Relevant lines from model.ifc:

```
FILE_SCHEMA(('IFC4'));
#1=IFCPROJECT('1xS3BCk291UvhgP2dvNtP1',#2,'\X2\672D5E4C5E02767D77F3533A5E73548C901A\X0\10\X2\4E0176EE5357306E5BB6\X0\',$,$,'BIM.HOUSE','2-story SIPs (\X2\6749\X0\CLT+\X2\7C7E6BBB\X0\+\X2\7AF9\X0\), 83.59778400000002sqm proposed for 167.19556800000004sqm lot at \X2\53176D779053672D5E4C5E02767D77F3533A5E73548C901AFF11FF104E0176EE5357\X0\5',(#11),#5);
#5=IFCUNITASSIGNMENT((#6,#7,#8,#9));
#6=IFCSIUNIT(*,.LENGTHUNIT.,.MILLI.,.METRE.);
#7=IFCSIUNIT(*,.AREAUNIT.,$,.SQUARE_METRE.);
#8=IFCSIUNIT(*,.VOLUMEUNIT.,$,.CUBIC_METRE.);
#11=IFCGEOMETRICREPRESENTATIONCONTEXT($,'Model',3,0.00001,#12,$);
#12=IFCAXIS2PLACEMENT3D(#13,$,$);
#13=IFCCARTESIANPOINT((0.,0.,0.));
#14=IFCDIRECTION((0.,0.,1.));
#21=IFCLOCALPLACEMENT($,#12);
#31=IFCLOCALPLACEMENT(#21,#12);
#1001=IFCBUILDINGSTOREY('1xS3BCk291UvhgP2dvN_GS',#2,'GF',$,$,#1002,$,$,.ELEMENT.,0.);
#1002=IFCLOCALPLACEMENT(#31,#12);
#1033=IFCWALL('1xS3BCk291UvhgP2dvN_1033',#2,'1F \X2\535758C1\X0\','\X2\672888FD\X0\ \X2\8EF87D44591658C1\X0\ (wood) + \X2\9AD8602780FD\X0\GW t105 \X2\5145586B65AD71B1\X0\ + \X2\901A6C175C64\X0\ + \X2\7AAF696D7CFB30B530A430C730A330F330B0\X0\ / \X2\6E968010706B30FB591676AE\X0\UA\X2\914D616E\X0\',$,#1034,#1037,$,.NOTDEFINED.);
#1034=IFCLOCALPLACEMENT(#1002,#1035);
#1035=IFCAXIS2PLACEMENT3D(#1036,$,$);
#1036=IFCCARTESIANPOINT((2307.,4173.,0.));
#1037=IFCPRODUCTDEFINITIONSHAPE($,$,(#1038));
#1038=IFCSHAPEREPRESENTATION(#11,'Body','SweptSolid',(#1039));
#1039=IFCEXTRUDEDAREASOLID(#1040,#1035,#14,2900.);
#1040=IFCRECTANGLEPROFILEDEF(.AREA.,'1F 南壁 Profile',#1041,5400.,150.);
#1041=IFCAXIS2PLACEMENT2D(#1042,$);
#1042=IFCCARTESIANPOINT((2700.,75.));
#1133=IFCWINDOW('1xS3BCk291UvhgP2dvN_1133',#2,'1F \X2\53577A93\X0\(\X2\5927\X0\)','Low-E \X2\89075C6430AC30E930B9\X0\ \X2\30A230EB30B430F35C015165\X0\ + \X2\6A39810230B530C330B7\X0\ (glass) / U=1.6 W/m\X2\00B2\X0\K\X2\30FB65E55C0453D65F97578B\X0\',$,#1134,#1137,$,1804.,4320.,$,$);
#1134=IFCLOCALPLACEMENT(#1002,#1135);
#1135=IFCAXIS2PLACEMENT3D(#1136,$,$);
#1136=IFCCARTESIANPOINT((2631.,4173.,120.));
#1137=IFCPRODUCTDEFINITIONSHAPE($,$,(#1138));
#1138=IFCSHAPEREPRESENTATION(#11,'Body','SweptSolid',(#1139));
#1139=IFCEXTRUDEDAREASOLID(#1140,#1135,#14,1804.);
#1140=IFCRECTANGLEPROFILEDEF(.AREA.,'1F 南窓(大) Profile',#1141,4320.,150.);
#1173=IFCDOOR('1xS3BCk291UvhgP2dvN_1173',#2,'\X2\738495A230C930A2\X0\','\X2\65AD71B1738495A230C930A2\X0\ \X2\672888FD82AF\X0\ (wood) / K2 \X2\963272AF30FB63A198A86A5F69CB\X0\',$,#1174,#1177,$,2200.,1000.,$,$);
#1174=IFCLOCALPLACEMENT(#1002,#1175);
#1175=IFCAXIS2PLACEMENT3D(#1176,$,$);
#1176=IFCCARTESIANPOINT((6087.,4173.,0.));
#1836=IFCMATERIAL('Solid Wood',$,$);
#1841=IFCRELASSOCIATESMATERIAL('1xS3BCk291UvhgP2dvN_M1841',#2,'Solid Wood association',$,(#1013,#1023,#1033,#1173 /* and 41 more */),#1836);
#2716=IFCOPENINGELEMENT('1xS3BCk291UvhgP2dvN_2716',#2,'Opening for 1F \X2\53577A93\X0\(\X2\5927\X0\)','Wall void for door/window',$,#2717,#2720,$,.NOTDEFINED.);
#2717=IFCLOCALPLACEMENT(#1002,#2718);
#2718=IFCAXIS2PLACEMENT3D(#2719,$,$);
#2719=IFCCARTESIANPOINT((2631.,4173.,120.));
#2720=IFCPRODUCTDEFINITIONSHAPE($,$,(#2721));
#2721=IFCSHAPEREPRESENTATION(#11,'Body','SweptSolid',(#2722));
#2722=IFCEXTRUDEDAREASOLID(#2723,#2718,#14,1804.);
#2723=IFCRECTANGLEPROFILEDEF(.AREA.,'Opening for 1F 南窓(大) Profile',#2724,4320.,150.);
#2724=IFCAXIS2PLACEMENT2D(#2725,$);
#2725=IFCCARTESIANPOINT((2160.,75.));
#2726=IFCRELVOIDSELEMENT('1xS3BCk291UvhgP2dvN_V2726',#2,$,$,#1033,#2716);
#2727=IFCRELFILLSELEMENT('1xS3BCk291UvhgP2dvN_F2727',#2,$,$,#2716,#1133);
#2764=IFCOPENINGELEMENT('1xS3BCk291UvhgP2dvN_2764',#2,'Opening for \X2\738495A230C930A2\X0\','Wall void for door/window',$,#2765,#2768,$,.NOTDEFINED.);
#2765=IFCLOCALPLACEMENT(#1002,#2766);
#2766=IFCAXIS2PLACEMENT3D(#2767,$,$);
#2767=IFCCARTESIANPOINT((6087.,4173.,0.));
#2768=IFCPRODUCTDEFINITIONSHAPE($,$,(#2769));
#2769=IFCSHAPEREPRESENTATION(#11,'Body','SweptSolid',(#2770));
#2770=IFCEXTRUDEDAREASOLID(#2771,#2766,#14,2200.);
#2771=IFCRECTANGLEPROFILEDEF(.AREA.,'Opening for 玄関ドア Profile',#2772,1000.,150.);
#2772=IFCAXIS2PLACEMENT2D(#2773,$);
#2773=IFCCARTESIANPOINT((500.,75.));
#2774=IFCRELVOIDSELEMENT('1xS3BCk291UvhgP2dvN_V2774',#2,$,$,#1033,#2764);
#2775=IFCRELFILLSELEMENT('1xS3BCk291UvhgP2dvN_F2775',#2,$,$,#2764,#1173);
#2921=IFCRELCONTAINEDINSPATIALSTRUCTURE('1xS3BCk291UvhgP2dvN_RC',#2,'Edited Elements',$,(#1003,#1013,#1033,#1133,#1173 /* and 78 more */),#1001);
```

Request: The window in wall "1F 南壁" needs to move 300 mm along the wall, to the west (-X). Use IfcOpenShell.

```python
import ifcopenshell
import ifcopenshell.api.geometry
import ifcopenshell.util.placement
import ifcopenshell.util.unit

model = ifcopenshell.open("model.ifc")
unit_scale = ifcopenshell.util.unit.calculate_unit_scale(model)

window = model.by_guid("1xS3BCk291UvhgP2dvN_1133")
opening = window.FillsVoids[0].RelatingOpeningElement
wall = opening.VoidsElements[0].RelatingBuildingElement

wall_matrix = ifcopenshell.util.placement.get_local_placement(wall.ObjectPlacement)
shift = wall_matrix[:3, 0] * -0.3 / unit_scale
before = ifcopenshell.util.placement.get_local_placement(window.ObjectPlacement)[:3, 3].copy()

# The window is not placed relative to its opening, so move both.
for product in (opening, window):
    matrix = ifcopenshell.util.placement.get_local_placement(product.ObjectPlacement)
    matrix[:3, 3] += shift
    ifcopenshell.api.geometry.edit_object_placement(model, product=product, matrix=matrix, is_si=False)

after = ifcopenshell.util.placement.get_local_placement(window.ObjectPlacement)[:3, 3]
print("window moved by", (after - before).round(3) + 0.0)

model.write("model-out.ifc")
```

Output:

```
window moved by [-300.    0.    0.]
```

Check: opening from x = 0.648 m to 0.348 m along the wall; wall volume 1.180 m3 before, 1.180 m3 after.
